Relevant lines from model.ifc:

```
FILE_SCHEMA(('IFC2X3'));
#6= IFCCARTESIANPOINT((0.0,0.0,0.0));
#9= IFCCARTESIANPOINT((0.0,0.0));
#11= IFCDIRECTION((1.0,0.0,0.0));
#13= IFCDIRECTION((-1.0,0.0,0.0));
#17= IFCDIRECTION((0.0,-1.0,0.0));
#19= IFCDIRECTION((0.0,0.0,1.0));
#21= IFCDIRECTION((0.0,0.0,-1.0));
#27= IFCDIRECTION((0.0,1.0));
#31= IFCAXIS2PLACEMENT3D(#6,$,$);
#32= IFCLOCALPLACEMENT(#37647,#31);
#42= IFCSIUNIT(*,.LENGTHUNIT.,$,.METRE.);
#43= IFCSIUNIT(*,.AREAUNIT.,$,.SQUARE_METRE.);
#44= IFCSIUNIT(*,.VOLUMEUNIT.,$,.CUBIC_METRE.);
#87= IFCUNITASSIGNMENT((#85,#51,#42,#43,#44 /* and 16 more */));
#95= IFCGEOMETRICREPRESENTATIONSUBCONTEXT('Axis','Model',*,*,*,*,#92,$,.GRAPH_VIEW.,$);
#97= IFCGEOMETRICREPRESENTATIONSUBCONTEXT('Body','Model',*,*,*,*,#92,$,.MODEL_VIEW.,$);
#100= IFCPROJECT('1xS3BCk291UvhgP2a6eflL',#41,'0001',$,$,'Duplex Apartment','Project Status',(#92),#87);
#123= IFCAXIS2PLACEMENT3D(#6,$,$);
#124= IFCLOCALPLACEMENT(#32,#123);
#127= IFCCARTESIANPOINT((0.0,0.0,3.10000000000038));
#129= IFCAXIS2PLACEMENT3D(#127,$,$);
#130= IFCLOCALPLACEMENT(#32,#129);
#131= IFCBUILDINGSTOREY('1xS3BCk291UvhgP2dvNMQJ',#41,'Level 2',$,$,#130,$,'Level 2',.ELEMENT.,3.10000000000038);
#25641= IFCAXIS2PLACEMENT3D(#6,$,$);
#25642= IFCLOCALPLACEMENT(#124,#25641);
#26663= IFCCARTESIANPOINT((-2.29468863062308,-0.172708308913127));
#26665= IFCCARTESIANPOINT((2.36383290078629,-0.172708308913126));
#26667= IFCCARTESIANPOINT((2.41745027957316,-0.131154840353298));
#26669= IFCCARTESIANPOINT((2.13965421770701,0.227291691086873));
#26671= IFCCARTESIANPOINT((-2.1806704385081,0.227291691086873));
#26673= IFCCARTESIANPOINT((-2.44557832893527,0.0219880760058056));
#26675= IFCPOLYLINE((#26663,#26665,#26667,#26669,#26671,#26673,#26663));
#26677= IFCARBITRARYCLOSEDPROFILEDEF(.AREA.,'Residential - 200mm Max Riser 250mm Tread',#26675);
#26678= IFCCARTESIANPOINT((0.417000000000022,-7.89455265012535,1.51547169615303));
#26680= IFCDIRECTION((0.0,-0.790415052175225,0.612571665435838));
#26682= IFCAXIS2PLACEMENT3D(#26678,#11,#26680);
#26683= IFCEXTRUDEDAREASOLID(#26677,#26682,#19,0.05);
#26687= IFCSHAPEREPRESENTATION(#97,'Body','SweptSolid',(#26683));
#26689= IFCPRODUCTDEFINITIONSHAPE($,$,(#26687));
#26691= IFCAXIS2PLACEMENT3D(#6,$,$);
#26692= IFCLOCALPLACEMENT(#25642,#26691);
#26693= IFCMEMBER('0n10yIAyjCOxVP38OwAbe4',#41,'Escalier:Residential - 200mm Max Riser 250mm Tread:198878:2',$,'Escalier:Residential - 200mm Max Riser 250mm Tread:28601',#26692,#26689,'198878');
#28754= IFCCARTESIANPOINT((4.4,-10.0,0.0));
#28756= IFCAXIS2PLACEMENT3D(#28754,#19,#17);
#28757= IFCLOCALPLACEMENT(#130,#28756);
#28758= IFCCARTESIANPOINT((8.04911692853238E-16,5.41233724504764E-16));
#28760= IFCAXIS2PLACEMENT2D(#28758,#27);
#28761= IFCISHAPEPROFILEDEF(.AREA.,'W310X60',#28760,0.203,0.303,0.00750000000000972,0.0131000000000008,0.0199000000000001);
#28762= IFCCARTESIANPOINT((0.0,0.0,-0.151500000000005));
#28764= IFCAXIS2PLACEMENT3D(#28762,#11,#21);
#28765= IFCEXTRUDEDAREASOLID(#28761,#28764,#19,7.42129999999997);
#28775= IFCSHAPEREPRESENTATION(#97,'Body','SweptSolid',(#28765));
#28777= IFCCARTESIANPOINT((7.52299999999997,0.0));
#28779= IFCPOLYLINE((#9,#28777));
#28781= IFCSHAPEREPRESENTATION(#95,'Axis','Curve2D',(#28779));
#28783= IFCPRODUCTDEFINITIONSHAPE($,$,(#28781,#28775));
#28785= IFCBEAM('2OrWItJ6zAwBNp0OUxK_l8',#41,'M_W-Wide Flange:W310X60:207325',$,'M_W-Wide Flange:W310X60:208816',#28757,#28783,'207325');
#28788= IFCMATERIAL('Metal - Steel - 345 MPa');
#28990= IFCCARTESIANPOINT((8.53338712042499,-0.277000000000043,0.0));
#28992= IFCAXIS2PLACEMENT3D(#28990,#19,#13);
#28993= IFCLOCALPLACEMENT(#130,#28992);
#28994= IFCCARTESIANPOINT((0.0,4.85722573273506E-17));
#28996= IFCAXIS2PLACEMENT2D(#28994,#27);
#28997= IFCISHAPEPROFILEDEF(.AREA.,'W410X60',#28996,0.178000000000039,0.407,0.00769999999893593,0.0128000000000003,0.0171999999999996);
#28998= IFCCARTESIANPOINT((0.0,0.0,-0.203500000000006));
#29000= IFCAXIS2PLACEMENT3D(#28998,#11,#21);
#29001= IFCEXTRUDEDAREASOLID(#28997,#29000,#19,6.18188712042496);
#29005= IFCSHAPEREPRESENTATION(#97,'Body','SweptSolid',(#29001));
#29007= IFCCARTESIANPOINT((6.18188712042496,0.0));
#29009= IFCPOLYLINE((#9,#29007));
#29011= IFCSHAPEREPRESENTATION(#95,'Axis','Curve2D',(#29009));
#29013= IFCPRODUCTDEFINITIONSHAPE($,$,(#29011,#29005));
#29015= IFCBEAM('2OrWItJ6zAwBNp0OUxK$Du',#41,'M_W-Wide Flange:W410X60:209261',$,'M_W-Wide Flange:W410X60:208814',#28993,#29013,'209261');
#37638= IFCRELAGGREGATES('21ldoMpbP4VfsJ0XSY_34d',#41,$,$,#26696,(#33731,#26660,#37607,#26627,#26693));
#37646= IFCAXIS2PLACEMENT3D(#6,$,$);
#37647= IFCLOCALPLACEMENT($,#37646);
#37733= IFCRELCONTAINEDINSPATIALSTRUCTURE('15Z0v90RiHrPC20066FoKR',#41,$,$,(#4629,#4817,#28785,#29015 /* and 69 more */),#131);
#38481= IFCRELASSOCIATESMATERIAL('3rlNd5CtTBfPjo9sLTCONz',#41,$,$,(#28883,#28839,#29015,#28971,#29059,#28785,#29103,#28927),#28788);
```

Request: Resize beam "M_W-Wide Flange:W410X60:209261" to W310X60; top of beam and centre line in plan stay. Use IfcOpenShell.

```python
import ifcopenshell
import ifcopenshell.util.element
import ifcopenshell.util.representation

model = ifcopenshell.open("model.ifc")

member = model.by_guid("2OrWItJ6zAwBNp0OUxK$Du")
source = next(p for p in model.by_type("IfcIShapeProfileDef") if p.ProfileName == "W310X60")

body = ifcopenshell.util.representation.get_representation(member, "Model", "Body")
solid = body.Items[0]
old_profile = solid.SweptArea

# Copy the section's sizes but keep this member's own profile position.
profile = ifcopenshell.util.element.copy(model, source)
# Profiles are centred, so shift by half the change in depth to hold the top.
shift = (old_profile.OverallDepth - profile.OverallDepth) / 2
x, y = old_profile.Position.Location.Coordinates
up = (-1.0, 0.0)  # upwards, in the solid's own plane
location = model.createIfcCartesianPoint((x + up[0] * shift, y + up[1] * shift))
profile.Position = model.createIfcAxis2Placement2D(location, old_profile.Position.RefDirection)
solid.SweptArea = profile
if not model.get_total_inverses(old_profile):
    ifcopenshell.util.element.remove_deep2(model, old_profile)
member.Name = member.Name.replace("W410X60", "W310X60")
member.ObjectType = member.ObjectType.replace("W410X60", "W310X60")

print(solid.SweptArea)

model.write("model_edited.ifc")
```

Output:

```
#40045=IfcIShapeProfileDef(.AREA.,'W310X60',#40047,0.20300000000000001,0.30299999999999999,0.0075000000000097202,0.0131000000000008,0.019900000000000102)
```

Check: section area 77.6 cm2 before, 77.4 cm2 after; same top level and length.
